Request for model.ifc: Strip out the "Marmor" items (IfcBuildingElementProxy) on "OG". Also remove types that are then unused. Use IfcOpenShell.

First a look at what the model holds.

```python
import ifcopenshell
import ifcopenshell.util.element

model = ifcopenshell.open("model.ifc")
print(model.schema)
storey = next(s for s in model.by_type("IfcBuildingStorey") if s.Name == "OG")
proxies = [e for e in ifcopenshell.util.element.get_decomposition(storey) if e.is_a("IfcBuildingElementProxy")]
seen = {}
for e in proxies:
    element_type = ifcopenshell.util.element.get_type(e)
    name = element_type.Name if element_type not in (None, e) else None
    seen[name] = seen.get(name, 0) + 1
for name, count in sorted(seen.items(), key=str):
    print(count, "x", name)
```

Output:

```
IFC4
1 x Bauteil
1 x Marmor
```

```python
import ifcopenshell
import ifcopenshell.api.root
import ifcopenshell.util.element

model = ifcopenshell.open("model.ifc")

storey = next(s for s in model.by_type("IfcBuildingStorey") if s.Name == "OG")
proxies = [e for e in ifcopenshell.util.element.get_decomposition(storey) if e.is_a("IfcBuildingElementProxy")]
targets = [e for e in proxies if (t := ifcopenshell.util.element.get_type(e)) not in (None, e) and t.Name == "Marmor"]
types = {ifcopenshell.util.element.get_type(e) for e in targets} - {None, *targets}

for e in targets:
    ifcopenshell.api.root.remove_product(model, product=e)
print(len(targets), "removed")

unused = [t for t in types if not ifcopenshell.util.element.get_types(t)]
for t in unused:
    ifcopenshell.api.root.remove_product(model, product=t)
print(len(unused), "unused types removed")

model.write("model-out.ifc")
```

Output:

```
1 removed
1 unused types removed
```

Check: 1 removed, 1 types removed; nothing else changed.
